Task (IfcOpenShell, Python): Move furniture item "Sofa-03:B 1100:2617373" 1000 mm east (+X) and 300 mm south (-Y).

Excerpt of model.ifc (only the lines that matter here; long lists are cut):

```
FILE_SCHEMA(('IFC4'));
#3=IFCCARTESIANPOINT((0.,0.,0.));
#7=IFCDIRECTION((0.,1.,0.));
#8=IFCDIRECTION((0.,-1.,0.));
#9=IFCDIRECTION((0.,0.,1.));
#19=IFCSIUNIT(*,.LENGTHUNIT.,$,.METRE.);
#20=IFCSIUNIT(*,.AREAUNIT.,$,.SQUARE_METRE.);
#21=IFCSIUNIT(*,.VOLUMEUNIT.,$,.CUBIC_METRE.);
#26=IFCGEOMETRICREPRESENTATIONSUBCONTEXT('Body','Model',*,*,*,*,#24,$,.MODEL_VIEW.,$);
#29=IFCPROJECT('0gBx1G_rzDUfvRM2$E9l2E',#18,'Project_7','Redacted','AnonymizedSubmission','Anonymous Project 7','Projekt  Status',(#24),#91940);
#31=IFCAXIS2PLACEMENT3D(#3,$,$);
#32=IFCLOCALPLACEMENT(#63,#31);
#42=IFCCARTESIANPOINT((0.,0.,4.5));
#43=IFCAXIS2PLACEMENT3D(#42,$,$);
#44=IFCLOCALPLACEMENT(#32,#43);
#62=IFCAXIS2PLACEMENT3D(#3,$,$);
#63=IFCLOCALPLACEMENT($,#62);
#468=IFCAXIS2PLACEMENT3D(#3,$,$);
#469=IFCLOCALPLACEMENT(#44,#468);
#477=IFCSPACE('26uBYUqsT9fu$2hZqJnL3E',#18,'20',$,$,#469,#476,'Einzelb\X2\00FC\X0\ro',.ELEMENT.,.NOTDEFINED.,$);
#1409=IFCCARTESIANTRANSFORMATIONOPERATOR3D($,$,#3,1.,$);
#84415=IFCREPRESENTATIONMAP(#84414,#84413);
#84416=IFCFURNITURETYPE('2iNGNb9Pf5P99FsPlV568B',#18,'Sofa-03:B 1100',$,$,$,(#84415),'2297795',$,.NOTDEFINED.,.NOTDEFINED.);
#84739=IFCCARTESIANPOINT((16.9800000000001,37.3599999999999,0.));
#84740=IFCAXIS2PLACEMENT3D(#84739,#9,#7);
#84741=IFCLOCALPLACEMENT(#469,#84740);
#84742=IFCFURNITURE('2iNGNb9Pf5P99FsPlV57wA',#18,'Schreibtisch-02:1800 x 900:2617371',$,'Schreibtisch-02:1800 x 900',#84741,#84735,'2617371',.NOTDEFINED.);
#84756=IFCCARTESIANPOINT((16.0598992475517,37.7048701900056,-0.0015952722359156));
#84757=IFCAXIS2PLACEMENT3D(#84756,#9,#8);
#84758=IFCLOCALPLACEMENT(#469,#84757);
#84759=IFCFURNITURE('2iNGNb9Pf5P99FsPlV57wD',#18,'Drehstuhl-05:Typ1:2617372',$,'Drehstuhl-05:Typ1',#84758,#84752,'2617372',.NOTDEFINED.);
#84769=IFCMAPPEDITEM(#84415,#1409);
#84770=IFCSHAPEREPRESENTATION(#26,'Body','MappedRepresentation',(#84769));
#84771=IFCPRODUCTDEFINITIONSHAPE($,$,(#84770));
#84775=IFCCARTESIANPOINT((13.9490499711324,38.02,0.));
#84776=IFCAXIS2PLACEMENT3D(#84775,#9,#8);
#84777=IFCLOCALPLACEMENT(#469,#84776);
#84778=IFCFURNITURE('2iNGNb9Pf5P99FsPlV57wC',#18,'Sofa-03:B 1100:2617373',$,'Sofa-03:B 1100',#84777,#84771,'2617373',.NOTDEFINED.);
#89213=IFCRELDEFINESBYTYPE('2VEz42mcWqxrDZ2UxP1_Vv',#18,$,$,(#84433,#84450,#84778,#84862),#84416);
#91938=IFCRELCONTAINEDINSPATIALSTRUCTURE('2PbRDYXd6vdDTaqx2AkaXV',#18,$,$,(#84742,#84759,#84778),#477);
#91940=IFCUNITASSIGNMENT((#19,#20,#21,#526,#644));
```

```python
import ifcopenshell
import ifcopenshell.api.geometry
import ifcopenshell.util.placement

model = ifcopenshell.open("model.ifc")

item = model.by_guid("2iNGNb9Pf5P99FsPlV57wC")
matrix = ifcopenshell.util.placement.get_local_placement(item.ObjectPlacement)
matrix[0, 3] += 1.0
matrix[1, 3] -= 0.3
ifcopenshell.api.geometry.edit_object_placement(model, product=item, matrix=matrix, is_si=False)

print(ifcopenshell.util.placement.get_local_placement(item.ObjectPlacement).round(3) + 0.0)

model.write("model-out.ifc")
```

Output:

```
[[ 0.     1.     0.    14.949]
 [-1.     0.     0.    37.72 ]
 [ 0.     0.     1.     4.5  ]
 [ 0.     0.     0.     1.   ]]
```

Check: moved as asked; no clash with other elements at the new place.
